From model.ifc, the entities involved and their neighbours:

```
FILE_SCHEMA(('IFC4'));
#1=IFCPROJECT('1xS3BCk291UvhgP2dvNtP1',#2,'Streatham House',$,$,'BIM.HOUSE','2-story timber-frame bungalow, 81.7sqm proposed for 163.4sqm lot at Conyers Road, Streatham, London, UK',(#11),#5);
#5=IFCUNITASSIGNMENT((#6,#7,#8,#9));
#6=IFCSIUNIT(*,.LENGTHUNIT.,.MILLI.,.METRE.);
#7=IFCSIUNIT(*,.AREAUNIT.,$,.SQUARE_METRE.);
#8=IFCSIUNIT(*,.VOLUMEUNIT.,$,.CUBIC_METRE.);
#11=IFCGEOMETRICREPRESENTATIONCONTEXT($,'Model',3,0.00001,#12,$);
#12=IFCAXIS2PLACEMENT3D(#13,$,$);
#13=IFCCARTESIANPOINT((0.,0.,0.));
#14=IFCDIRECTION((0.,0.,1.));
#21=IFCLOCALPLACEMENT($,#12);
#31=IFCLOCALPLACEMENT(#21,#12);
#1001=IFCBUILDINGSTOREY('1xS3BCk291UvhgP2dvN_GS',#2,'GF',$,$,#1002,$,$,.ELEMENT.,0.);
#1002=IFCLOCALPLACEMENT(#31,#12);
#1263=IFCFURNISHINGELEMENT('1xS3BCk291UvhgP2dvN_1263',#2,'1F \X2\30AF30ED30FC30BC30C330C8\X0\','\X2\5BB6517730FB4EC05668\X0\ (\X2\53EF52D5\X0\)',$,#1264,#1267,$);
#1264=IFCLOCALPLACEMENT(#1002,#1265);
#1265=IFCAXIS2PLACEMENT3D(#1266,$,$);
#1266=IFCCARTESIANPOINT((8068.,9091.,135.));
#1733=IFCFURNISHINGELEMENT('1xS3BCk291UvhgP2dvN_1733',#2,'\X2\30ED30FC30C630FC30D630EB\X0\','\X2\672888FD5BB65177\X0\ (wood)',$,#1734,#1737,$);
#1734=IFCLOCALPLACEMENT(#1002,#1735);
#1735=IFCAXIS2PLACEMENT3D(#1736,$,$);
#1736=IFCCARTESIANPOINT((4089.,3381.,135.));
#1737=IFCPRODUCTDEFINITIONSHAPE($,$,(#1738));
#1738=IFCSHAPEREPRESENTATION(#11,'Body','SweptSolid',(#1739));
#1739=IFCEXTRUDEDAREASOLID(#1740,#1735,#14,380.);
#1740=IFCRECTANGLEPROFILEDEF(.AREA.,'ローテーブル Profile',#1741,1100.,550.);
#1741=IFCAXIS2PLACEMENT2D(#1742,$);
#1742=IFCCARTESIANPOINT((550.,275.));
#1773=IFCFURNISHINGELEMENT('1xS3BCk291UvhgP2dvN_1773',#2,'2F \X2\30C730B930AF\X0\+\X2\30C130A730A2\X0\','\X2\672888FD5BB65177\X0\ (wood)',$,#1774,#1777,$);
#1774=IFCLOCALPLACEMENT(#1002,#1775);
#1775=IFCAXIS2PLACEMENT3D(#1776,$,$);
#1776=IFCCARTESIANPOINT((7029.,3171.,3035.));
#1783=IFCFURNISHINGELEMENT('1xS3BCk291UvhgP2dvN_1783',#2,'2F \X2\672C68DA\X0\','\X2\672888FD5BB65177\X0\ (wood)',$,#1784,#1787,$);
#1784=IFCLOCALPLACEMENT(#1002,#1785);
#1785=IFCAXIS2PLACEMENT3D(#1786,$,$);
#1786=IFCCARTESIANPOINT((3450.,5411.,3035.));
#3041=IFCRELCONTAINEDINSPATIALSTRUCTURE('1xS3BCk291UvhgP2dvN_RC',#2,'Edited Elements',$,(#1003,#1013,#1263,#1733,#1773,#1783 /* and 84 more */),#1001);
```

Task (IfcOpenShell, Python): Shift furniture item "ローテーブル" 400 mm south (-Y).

```python
import ifcopenshell
import ifcopenshell.api.geometry
import ifcopenshell.util.placement
import ifcopenshell.util.unit

model = ifcopenshell.open("model.ifc")
unit_scale = ifcopenshell.util.unit.calculate_unit_scale(model)

item = model.by_id(1733)
matrix = ifcopenshell.util.placement.get_local_placement(item.ObjectPlacement)
matrix[1, 3] -= 0.4 / unit_scale
ifcopenshell.api.geometry.edit_object_placement(model, product=item, matrix=matrix, is_si=False)

print(ifcopenshell.util.placement.get_local_placement(item.ObjectPlacement).round(3) + 0.0)

model.write("model_rev.ifc")
```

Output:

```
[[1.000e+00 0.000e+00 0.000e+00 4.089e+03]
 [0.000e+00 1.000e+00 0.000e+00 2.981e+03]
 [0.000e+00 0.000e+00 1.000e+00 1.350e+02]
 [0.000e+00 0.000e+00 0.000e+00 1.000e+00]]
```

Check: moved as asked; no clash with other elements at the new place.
